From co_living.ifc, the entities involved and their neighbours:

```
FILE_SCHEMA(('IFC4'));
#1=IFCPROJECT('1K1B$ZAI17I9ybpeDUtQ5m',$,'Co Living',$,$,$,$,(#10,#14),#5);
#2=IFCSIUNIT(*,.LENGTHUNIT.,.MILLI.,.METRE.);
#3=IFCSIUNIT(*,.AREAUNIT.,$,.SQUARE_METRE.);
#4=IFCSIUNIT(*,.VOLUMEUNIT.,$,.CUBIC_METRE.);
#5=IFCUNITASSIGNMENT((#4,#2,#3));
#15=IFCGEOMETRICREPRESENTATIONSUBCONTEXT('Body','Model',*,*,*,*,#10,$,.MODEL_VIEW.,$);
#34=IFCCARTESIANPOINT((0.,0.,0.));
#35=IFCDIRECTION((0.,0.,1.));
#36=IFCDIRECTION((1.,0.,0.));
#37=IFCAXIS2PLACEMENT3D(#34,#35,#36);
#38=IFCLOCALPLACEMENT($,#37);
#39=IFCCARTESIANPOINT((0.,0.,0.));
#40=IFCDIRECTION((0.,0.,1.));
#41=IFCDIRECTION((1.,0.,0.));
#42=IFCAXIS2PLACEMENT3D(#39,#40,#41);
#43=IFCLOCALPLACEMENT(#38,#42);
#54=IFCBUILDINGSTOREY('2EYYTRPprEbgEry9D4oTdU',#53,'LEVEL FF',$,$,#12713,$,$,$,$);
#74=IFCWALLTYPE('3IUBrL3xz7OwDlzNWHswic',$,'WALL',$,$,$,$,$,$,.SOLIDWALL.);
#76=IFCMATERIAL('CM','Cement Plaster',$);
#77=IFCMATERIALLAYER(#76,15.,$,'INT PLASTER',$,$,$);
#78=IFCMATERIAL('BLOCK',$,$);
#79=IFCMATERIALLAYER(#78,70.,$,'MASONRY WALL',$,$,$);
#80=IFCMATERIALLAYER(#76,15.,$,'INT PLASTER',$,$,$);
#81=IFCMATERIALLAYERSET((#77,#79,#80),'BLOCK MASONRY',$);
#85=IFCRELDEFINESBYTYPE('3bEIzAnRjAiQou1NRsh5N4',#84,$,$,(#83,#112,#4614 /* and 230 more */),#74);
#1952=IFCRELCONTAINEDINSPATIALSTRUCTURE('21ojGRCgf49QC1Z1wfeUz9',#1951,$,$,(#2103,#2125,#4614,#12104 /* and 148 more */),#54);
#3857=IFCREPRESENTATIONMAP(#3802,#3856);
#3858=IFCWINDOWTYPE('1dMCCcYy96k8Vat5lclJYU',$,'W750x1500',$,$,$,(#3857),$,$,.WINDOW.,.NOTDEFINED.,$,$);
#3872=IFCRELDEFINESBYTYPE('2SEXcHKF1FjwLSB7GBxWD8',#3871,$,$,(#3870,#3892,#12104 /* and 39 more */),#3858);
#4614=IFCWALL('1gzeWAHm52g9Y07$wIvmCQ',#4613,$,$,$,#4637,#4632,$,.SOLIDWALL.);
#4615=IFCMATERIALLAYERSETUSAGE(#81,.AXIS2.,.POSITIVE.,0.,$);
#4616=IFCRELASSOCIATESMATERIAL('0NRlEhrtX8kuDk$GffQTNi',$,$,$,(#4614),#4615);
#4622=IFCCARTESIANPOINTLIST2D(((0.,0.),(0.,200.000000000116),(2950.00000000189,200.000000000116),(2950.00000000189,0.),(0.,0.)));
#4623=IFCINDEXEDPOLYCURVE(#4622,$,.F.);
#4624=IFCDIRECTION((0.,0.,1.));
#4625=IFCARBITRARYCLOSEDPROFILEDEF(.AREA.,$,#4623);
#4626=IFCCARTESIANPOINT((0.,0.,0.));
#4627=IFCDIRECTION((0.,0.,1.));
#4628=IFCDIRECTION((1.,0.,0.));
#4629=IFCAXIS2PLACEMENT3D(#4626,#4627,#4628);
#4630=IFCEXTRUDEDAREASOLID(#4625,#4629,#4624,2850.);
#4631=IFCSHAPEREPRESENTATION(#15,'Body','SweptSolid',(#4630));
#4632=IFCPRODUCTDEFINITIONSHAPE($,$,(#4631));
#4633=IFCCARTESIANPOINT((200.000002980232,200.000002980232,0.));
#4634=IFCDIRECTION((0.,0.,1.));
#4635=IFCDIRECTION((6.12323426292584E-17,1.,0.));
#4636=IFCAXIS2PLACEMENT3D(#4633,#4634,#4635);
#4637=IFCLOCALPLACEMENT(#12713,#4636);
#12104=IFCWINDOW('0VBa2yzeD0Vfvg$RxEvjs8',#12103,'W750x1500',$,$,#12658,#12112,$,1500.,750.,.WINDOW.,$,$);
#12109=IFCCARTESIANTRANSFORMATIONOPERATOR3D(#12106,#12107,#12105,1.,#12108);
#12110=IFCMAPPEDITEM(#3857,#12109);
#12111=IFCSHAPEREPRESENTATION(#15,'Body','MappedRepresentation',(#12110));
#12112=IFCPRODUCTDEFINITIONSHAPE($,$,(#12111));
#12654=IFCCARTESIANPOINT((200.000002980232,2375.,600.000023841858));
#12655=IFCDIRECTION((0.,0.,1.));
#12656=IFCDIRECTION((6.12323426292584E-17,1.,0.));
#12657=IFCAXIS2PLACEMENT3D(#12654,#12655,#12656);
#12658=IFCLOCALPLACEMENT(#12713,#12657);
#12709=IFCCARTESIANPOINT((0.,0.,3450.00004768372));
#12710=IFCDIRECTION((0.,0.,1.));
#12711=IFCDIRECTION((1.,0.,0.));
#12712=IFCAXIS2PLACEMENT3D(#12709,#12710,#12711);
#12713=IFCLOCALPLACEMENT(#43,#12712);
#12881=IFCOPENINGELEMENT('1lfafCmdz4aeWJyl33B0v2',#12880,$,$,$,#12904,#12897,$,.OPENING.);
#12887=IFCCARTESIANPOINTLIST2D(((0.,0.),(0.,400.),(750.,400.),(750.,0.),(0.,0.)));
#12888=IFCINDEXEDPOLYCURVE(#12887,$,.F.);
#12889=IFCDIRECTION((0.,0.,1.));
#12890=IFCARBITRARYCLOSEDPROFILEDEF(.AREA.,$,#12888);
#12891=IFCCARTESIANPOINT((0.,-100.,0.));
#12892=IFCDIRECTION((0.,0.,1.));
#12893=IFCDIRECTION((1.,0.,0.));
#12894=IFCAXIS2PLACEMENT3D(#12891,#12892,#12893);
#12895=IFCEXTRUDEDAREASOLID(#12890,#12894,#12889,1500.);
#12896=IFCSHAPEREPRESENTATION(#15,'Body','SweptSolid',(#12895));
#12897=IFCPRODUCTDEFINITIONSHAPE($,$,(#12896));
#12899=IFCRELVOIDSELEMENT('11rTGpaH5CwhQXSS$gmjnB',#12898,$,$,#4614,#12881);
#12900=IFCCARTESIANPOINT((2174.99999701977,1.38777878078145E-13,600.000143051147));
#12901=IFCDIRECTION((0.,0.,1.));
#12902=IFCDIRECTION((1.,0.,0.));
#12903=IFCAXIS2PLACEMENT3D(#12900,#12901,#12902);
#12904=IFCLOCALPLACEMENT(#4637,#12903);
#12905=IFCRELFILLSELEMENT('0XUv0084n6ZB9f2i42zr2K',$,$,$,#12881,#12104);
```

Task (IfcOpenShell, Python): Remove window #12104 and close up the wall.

```python
import ifcopenshell
import ifcopenshell.api.feature
import ifcopenshell.api.root
import ifcopenshell.geom
import ifcopenshell.util.shape

model = ifcopenshell.open("co_living.ifc")
settings = ifcopenshell.geom.settings()


def volume(element):
    """Net volume in cubic metres, openings subtracted."""
    shape = ifcopenshell.geom.create_shape(settings, element)
    return ifcopenshell.util.shape.get_volume(shape.geometry)


window = model.by_guid("0VBa2yzeD0Vfvg$RxEvjs8")
opening = window.FillsVoids[0].RelatingOpeningElement
wall = opening.VoidsElements[0].RelatingBuildingElement
before = volume(wall)

ifcopenshell.api.root.remove_product(model, product=window)
ifcopenshell.api.feature.remove_feature(model, feature=opening)

after = volume(wall)

print(f"wall volume {before:.3f} -> {after:.3f} m3")

model.write("co_living_v2.ifc")
```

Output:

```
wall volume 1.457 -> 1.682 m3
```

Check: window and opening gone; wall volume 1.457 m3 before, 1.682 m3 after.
